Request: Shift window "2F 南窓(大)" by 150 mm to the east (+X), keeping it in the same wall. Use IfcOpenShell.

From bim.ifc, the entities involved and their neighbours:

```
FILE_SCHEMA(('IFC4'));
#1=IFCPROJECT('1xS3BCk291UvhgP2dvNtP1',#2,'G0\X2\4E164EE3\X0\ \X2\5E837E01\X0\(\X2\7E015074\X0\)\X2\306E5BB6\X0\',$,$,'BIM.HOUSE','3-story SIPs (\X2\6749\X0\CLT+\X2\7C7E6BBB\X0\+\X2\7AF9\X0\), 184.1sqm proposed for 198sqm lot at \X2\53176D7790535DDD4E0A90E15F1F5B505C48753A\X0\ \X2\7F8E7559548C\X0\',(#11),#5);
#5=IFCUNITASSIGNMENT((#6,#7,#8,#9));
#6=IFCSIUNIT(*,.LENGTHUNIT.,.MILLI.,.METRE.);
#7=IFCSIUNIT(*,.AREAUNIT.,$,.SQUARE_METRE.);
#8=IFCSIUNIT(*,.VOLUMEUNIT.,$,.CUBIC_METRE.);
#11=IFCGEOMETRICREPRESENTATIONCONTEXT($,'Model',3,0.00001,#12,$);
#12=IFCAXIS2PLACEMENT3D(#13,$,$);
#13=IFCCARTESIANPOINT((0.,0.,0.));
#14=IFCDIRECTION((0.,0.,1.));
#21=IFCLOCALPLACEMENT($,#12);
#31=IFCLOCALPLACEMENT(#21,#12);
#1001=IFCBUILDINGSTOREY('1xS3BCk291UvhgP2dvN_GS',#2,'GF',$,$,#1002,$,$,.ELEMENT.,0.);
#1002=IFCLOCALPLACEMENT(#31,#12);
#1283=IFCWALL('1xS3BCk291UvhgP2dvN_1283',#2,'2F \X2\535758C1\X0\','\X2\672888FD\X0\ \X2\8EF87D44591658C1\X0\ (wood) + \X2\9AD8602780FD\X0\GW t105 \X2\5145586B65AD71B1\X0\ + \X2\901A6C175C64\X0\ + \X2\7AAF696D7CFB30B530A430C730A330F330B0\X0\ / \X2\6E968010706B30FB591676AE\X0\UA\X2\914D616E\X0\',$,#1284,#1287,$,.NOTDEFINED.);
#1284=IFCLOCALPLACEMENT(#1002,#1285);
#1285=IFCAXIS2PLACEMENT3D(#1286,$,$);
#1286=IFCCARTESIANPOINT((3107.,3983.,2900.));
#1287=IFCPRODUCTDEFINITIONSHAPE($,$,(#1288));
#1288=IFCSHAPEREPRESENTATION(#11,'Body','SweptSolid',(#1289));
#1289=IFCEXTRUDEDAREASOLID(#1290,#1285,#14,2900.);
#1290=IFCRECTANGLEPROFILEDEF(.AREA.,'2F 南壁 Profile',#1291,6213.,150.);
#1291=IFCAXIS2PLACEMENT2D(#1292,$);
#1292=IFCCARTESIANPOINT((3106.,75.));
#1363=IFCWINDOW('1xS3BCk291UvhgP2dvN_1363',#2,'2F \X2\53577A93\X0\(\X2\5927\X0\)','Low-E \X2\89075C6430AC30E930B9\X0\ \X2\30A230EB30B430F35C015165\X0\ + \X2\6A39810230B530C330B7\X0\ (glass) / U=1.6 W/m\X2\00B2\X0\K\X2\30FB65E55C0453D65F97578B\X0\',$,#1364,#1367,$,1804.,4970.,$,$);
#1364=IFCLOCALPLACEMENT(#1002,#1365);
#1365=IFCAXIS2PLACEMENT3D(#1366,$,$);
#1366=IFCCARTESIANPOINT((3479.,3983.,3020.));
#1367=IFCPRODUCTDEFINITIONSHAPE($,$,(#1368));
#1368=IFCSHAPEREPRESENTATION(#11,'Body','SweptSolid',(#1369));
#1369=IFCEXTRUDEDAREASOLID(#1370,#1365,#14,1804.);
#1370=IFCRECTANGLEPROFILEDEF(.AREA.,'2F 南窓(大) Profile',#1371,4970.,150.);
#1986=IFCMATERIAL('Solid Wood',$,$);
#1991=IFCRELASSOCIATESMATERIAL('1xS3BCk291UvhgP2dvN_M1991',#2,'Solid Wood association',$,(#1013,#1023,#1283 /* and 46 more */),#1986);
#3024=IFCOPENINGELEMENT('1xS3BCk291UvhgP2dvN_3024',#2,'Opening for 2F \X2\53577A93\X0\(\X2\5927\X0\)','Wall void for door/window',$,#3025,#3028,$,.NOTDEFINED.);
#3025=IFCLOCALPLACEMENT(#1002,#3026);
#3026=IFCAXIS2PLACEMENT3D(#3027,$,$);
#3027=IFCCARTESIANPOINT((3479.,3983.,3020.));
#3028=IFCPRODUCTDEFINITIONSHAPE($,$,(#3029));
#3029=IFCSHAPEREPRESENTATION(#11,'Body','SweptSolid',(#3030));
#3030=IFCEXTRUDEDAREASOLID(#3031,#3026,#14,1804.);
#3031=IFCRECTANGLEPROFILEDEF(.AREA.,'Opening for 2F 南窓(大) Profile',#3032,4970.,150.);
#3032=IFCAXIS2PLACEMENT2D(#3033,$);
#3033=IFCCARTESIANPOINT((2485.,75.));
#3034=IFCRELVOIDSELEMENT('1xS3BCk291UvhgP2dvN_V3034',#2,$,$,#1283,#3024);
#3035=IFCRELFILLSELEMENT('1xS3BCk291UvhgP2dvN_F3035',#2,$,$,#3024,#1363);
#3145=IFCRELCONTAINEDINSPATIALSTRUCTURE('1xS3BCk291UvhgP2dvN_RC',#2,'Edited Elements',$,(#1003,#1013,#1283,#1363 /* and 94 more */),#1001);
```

```python
import ifcopenshell
import ifcopenshell.api.geometry
import ifcopenshell.util.placement

model = ifcopenshell.open("bim.ifc")

window = model.by_guid("1xS3BCk291UvhgP2dvN_1363")
opening = window.FillsVoids[0].RelatingOpeningElement
wall = opening.VoidsElements[0].RelatingBuildingElement

wall_matrix = ifcopenshell.util.placement.get_local_placement(wall.ObjectPlacement)
shift = wall_matrix[:3, 0] * 150.0
before = ifcopenshell.util.placement.get_local_placement(window.ObjectPlacement)[:3, 3].copy()

# The window is not placed relative to its opening, so move both.
for product in (opening, window):
    matrix = ifcopenshell.util.placement.get_local_placement(product.ObjectPlacement)
    matrix[:3, 3] += shift
    ifcopenshell.api.geometry.edit_object_placement(model, product=product, matrix=matrix, is_si=False)

after = ifcopenshell.util.placement.get_local_placement(window.ObjectPlacement)[:3, 3]
print("window moved by", (after - before).round(3) + 0.0)

model.write("bim_updated.ifc")
```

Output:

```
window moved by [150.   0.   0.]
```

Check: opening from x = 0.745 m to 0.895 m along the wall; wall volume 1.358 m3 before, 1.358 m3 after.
